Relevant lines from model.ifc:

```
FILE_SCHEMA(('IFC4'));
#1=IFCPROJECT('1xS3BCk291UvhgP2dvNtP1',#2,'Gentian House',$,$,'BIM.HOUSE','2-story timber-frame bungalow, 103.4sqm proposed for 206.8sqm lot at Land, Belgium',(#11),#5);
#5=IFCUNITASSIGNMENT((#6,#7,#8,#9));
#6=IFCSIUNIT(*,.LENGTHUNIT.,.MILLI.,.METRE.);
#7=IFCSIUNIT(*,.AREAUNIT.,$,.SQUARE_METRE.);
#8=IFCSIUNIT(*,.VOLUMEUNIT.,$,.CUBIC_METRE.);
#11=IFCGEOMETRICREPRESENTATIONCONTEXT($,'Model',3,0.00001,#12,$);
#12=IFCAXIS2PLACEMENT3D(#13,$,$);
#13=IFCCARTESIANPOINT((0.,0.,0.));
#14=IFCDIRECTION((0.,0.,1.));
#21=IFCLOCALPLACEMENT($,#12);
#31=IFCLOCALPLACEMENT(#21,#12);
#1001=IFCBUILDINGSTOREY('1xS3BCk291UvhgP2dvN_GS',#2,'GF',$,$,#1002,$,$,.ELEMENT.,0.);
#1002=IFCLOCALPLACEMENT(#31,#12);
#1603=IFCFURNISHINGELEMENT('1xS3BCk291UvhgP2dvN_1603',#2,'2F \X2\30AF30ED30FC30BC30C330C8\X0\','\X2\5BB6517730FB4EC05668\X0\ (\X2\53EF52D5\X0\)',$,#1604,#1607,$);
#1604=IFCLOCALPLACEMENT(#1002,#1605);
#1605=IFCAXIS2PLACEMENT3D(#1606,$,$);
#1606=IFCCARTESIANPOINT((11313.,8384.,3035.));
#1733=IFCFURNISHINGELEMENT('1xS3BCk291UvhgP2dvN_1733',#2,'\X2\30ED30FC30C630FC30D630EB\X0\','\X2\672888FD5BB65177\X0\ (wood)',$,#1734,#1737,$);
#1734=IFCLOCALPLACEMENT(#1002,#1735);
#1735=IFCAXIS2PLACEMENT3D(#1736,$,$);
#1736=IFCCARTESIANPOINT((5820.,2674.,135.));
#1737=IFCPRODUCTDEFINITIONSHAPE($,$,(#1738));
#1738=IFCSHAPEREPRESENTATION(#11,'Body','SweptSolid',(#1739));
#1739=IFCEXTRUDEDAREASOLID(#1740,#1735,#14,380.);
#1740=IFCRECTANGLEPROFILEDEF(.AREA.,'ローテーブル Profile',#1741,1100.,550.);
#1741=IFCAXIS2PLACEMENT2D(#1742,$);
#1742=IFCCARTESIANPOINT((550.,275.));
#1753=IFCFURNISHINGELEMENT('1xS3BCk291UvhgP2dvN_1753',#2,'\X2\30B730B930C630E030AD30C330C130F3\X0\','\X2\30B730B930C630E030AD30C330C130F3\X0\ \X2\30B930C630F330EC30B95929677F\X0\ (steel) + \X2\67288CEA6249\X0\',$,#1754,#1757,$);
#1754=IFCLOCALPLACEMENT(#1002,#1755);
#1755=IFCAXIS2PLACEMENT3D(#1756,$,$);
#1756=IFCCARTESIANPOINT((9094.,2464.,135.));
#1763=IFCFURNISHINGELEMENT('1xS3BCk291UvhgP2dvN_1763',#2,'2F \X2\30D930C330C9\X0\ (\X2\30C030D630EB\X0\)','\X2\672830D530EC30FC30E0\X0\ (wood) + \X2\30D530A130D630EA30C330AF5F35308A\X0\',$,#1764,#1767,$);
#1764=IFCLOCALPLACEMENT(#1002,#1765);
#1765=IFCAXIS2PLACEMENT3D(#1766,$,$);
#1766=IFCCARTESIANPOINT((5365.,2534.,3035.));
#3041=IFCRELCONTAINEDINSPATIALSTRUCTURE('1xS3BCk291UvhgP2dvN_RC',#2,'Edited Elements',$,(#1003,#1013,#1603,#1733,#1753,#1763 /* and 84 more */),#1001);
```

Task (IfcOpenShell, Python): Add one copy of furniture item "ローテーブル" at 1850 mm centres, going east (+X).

```python
import numpy as np
import ifcopenshell
import ifcopenshell.api.geometry
import ifcopenshell.api.root
import ifcopenshell.util.element
import ifcopenshell.util.placement
import ifcopenshell.util.unit

model = ifcopenshell.open("model.ifc")
unit_scale = ifcopenshell.util.unit.calculate_unit_scale(model)


def reuse_history(source, copy):
    """copy_class also copies each property set's owner history, people and application; keep the originals."""
    for rel in copy.IsDefinedBy:
        if rel.is_a("IfcRelDefinesByProperties") and (history := rel.RelatingPropertyDefinition.OwnerHistory):
            rel.RelatingPropertyDefinition.OwnerHistory = source.OwnerHistory
            ifcopenshell.util.element.remove_deep2(model, history)


source = model.by_guid("1xS3BCk291UvhgP2dvN_1733")
base = ifcopenshell.util.placement.get_local_placement(source.ObjectPlacement)
step = np.array([1.0, 0.0, 0.0]) * 1.85 / unit_scale

for i in range(1, 2):
    copy = ifcopenshell.api.root.copy_class(model, product=source)
    copy.Representation = ifcopenshell.util.element.copy_deep(
        model, source.Representation, exclude=["IfcGeometricRepresentationContext", "IfcRepresentationMap"]
    )
    reuse_history(source, copy)
    matrix = base.copy()
    matrix[:3, 3] += i * step
    print("added at", matrix[:3, 3].round(3) + 0.0)
    ifcopenshell.api.geometry.edit_object_placement(model, product=copy, matrix=matrix, is_si=False)

model.write("model_edited.ifc")
```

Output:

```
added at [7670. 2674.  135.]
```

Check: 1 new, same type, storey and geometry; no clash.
